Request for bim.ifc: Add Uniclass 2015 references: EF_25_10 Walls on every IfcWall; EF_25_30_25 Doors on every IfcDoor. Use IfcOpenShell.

First a look at what the model holds.

```python
import ifcopenshell

model = ifcopenshell.open("bim.ifc")
print(model.schema)
print("classifications:", [c.Name for c in model.by_type("IfcClassification")])
for ifc_class in ("IfcDoor", "IfcRoof", "IfcStair", "IfcWall", "IfcWindow"):
    print(ifc_class, len(model.by_type(ifc_class)))
```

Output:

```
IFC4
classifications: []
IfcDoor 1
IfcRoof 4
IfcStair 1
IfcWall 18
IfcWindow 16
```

```python
import ifcopenshell
import ifcopenshell.api.classification

model = ifcopenshell.open("bim.ifc")

system = ifcopenshell.api.classification.add_classification(model, classification="Uniclass 2015")

codes = {
    "IfcWall": ("EF_25_10", "Walls"),
    "IfcDoor": ("EF_25_30_25", "Doors"),
}
for ifc_class, (code, name) in codes.items():
    products = model.by_type(ifc_class)
    ifcopenshell.api.classification.add_reference(
        model, products=products, classification=system, identification=code, name=name
    )
    print(code, len(products))

model.write("bim-out.ifc")
```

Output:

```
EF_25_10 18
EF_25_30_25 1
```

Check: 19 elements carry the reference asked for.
